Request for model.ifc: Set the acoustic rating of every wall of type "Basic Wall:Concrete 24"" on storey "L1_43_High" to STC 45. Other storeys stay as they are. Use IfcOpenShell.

First a look at what the model holds.

```python
import ifcopenshell
import ifcopenshell.util.element

model = ifcopenshell.open("model.ifc")
print(model.schema)
storey = next(s for s in model.by_type("IfcBuildingStorey") if s.Name == "L1_43_High")
walls = [e for e in ifcopenshell.util.element.get_decomposition(storey) if e.is_a("IfcWall")]
seen = {}
for e in walls:
    element_type = ifcopenshell.util.element.get_type(e)
    key = (element_type.Name if element_type != e and element_type else None, ifcopenshell.util.element.get_pset(e, "Pset_WallCommon", "AcousticRating"))
    seen[key] = seen.get(key, 0) + 1
for (name, value), count in sorted(seen.items(), key=str):
    print(count, "x", name, "|", value)
```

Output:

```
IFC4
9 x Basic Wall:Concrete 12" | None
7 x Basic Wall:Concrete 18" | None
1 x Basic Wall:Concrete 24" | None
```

```python
import ifcopenshell
import ifcopenshell.api.pset
import ifcopenshell.util.element

model = ifcopenshell.open("model.ifc")

storey = next(s for s in model.by_type("IfcBuildingStorey") if s.Name == "L1_43_High")
walls = [e for e in ifcopenshell.util.element.get_decomposition(storey) if e.is_a("IfcWall")]

count = 0
for e in walls:
    element_type = ifcopenshell.util.element.get_type(e)
    if element_type in (None, e) or element_type.Name != 'Basic Wall:Concrete 24"':
        continue
    # add_pset returns the element's existing set when there is one.
    pset = ifcopenshell.api.pset.add_pset(model, product=e, name="Pset_WallCommon")
    ifcopenshell.api.pset.edit_pset(model, pset=pset, properties={"AcousticRating": "STC 45"})
    count += 1

print(count, "walls updated")

model.write("model_rev.ifc")
```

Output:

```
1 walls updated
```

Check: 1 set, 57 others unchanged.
